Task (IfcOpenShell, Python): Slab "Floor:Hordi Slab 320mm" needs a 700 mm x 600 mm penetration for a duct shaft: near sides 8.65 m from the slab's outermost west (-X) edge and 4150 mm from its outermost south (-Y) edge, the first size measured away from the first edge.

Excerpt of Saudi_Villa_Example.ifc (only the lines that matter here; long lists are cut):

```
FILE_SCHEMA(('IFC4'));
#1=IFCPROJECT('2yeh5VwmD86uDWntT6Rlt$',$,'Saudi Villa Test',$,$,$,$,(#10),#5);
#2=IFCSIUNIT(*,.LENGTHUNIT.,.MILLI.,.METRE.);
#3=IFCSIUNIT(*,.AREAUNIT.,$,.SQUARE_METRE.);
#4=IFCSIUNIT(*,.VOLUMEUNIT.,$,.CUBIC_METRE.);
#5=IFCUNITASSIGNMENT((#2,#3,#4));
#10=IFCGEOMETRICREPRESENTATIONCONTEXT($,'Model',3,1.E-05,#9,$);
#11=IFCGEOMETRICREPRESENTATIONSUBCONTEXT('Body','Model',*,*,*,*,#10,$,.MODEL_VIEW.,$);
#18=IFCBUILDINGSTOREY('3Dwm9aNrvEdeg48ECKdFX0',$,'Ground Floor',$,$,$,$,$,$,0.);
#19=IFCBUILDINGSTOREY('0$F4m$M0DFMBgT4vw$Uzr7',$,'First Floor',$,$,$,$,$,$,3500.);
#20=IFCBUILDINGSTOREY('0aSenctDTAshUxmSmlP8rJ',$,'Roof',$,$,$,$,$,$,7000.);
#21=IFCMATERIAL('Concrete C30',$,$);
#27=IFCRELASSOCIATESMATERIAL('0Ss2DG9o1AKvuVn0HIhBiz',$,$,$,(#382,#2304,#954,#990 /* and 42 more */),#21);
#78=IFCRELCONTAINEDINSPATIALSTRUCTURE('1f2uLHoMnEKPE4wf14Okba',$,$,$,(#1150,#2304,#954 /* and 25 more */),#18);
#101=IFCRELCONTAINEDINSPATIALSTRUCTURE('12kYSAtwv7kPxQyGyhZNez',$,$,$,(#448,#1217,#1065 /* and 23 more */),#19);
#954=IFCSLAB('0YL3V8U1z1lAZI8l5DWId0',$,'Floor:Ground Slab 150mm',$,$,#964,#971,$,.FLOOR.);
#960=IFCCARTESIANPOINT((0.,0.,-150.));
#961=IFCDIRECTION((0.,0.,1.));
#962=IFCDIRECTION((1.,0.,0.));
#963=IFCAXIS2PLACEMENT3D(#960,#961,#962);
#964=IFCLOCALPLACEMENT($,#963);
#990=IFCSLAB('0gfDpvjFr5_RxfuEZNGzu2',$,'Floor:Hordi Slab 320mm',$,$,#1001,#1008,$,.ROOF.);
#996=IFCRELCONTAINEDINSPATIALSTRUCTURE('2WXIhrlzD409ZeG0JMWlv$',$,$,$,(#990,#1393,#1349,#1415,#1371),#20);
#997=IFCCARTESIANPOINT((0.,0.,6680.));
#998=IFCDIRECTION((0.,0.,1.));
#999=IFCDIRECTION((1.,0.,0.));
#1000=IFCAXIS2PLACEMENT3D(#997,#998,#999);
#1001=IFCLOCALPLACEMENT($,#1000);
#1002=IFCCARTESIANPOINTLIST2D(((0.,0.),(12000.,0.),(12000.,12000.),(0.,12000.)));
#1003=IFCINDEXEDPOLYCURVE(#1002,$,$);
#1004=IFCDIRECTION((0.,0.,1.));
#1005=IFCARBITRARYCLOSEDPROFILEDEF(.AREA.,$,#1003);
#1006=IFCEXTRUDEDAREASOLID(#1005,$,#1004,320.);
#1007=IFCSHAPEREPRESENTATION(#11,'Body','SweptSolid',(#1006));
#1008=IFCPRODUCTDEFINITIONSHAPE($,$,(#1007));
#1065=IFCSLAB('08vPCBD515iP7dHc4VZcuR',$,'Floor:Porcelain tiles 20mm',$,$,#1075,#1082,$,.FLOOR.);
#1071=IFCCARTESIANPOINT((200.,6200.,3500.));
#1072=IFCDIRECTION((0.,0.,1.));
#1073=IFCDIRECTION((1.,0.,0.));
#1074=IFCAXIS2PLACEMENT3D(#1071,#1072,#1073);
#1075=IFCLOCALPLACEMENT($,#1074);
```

```python
import numpy as np
import ifcopenshell
import ifcopenshell.api.feature
import ifcopenshell.api.geometry
import ifcopenshell.api.root
import ifcopenshell.geom
import ifcopenshell.util.placement
import ifcopenshell.util.representation
import ifcopenshell.util.shape
import ifcopenshell.util.unit

model = ifcopenshell.open("Saudi_Villa_Example.ifc")
unit_scale = ifcopenshell.util.unit.calculate_unit_scale(model)
settings = ifcopenshell.geom.settings()


def volume(element):
    """Net volume in cubic metres, openings subtracted."""
    shape = ifcopenshell.geom.create_shape(settings, element)
    return ifcopenshell.util.shape.get_volume(shape.geometry)


slab = model.by_guid("0gfDpvjFr5_RxfuEZNGzu2")
before = volume(slab)

# Extent in the slab's own axes, in metres. The edges named are its -X and -Y sides.
slab_shape = ifcopenshell.geom.create_shape(settings, slab)
vertices = ifcopenshell.util.shape.get_vertices(slab_shape.geometry)
x_min, y_min, bottom = vertices.min(axis=0)
top = vertices[:, 2].max()

opening = ifcopenshell.api.root.create_entity(model, ifc_class="IfcOpeningElement", name="Duct shaft opening", predefined_type="OPENING")
context = ifcopenshell.util.representation.get_context(model, "Model", "Body", "MODEL_VIEW")
width, depth = 0.7, 0.6
outline = [(0.0, 0.0), (width, 0.0), (width, depth), (0.0, depth), (0.0, 0.0)]
# Overshoot both faces by 50 mm so the cut is clean.
shape = ifcopenshell.api.geometry.add_slab_representation(
    model, context=context, depth=top - bottom + 0.1, polyline=outline
)
ifcopenshell.api.geometry.assign_representation(model, product=opening, representation=shape)

matrix = ifcopenshell.util.placement.get_local_placement(slab.ObjectPlacement)
matrix[:, 3] = matrix @ np.append(np.array([x_min + 8.65, y_min + 4.15, bottom - 0.05]) / unit_scale, 1.0)
ifcopenshell.api.geometry.edit_object_placement(model, product=opening, matrix=matrix, is_si=False)
ifcopenshell.api.feature.add_feature(model, feature=opening, element=slab)

after = volume(slab)

print(f"slab volume {before:.3f} -> {after:.3f} m3")

model.write("Saudi_Villa_Example_rev.ifc")
```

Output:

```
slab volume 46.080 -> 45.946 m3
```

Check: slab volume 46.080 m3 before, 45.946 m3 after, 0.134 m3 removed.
